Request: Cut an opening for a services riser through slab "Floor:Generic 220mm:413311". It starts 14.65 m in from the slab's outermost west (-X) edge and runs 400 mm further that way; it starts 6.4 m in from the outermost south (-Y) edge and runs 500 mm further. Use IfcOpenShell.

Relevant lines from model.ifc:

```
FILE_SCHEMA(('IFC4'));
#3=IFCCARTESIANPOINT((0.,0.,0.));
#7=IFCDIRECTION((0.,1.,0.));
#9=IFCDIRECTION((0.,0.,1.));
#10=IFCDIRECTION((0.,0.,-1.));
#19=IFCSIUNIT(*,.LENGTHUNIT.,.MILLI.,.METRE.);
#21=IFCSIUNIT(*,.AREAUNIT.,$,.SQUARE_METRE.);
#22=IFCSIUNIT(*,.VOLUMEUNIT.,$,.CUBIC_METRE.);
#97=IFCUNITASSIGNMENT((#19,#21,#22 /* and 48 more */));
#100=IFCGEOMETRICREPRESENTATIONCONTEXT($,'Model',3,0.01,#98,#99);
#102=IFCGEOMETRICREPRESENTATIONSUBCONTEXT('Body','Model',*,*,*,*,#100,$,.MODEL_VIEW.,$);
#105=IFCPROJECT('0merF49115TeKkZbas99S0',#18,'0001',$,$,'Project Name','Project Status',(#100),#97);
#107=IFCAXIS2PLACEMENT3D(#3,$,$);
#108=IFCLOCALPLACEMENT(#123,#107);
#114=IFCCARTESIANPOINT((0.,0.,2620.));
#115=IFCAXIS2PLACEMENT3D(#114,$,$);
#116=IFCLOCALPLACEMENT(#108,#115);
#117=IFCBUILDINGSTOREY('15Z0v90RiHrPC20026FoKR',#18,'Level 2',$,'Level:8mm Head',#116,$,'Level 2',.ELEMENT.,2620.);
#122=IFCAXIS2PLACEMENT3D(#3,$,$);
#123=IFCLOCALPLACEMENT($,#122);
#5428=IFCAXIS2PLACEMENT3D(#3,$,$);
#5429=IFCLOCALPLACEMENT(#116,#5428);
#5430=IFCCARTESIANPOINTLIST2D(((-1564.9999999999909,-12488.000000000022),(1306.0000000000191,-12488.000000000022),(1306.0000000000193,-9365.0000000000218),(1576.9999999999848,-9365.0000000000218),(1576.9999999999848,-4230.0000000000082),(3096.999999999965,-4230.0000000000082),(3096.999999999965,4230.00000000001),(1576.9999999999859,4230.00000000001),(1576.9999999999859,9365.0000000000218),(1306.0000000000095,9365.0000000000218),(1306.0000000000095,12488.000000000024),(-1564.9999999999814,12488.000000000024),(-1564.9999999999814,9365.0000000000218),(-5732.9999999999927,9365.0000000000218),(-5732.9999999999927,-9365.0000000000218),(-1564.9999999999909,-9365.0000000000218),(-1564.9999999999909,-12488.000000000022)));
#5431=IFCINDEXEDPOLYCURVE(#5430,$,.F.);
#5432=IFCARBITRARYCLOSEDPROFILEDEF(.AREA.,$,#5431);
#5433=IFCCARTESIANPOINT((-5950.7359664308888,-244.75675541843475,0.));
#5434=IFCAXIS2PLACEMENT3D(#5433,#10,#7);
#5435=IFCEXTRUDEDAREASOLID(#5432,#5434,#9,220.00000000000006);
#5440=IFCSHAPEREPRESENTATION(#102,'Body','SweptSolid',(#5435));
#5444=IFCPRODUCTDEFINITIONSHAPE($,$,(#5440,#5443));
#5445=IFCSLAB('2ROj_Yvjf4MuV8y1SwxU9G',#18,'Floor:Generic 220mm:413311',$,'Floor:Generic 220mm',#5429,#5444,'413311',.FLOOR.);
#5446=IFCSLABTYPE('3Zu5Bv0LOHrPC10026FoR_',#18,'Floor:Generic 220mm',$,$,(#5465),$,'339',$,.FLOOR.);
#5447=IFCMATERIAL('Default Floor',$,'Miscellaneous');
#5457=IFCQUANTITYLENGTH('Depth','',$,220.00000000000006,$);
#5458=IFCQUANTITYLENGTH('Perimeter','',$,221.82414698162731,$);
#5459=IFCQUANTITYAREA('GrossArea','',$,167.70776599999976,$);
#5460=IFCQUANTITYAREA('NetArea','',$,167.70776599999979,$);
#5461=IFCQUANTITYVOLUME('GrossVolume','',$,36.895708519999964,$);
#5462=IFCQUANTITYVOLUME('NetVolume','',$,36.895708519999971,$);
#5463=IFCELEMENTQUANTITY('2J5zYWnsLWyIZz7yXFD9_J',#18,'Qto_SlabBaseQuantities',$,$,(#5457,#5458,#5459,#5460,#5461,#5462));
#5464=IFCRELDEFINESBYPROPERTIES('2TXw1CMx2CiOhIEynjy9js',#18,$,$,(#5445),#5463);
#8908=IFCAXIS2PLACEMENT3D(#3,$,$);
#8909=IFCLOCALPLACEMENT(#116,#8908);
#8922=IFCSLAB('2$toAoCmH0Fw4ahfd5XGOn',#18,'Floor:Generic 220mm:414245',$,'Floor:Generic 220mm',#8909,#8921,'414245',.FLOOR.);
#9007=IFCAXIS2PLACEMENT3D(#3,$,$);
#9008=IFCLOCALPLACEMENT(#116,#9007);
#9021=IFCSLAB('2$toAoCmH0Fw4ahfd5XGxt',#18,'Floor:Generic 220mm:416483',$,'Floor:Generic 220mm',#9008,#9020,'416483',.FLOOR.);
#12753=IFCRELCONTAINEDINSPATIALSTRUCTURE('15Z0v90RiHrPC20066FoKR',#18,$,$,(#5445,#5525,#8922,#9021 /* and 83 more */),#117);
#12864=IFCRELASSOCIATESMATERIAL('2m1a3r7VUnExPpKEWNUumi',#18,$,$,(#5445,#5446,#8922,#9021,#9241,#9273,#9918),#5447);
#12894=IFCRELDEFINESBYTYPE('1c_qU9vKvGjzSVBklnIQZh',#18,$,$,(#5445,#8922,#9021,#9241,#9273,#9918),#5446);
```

```python
import numpy as np
import ifcopenshell
import ifcopenshell.api.feature
import ifcopenshell.api.geometry
import ifcopenshell.api.pset
import ifcopenshell.api.root
import ifcopenshell.geom
import ifcopenshell.util.element
import ifcopenshell.util.placement
import ifcopenshell.util.representation
import ifcopenshell.util.shape
import ifcopenshell.util.unit

model = ifcopenshell.open("model.ifc")
unit_scale = ifcopenshell.util.unit.calculate_unit_scale(model)
area_scale = ifcopenshell.util.unit.calculate_unit_scale(model, "AREAUNIT")
volume_scale = ifcopenshell.util.unit.calculate_unit_scale(model, "VOLUMEUNIT")
settings = ifcopenshell.geom.settings()


def volume(element):
    """Net volume in cubic metres, openings subtracted."""
    shape = ifcopenshell.geom.create_shape(settings, element)
    return ifcopenshell.util.shape.get_volume(shape.geometry)


slab = model.by_guid("2ROj_Yvjf4MuV8y1SwxU9G")
before = volume(slab)

# Extent in the slab's own axes, in metres. The edges named are its -X and -Y sides.
slab_shape = ifcopenshell.geom.create_shape(settings, slab)
vertices = ifcopenshell.util.shape.get_vertices(slab_shape.geometry)
x_min, y_min, bottom = vertices.min(axis=0)
top = vertices[:, 2].max()

opening = ifcopenshell.api.root.create_entity(model, ifc_class="IfcOpeningElement", name="Services riser opening", predefined_type="OPENING")
context = ifcopenshell.util.representation.get_context(model, "Model", "Body", "MODEL_VIEW")
width, depth = 0.4, 0.5
outline = [(0.0, 0.0), (width, 0.0), (width, depth), (0.0, depth), (0.0, 0.0)]
# Overshoot both faces by 50 mm so the cut is clean.
shape = ifcopenshell.api.geometry.add_slab_representation(
    model, context=context, depth=top - bottom + 0.1, polyline=outline
)
ifcopenshell.api.geometry.assign_representation(model, product=opening, representation=shape)

matrix = ifcopenshell.util.placement.get_local_placement(slab.ObjectPlacement)
matrix[:, 3] = matrix @ np.append(np.array([x_min + 14.65, y_min + 6.4, bottom - 0.05]) / unit_scale, 1.0)
ifcopenshell.api.geometry.edit_object_placement(model, product=opening, matrix=matrix, is_si=False)
ifcopenshell.api.feature.add_feature(model, feature=opening, element=slab)

after = volume(slab)

# Update the slab's stored quantities.
qto = model.by_id(ifcopenshell.util.element.get_pset(slab, "Qto_SlabBaseQuantities", should_inherit=False)["id"])
ifcopenshell.api.pset.edit_qto(model, qto=qto, properties={
    "NetArea": after / (top - bottom) / area_scale,
    "NetVolume": after / volume_scale,
})

print(f"slab volume {before:.3f} -> {after:.3f} m3")

model.write("model_rev.ifc")
```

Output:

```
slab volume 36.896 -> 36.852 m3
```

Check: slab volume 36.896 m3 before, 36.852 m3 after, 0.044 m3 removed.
